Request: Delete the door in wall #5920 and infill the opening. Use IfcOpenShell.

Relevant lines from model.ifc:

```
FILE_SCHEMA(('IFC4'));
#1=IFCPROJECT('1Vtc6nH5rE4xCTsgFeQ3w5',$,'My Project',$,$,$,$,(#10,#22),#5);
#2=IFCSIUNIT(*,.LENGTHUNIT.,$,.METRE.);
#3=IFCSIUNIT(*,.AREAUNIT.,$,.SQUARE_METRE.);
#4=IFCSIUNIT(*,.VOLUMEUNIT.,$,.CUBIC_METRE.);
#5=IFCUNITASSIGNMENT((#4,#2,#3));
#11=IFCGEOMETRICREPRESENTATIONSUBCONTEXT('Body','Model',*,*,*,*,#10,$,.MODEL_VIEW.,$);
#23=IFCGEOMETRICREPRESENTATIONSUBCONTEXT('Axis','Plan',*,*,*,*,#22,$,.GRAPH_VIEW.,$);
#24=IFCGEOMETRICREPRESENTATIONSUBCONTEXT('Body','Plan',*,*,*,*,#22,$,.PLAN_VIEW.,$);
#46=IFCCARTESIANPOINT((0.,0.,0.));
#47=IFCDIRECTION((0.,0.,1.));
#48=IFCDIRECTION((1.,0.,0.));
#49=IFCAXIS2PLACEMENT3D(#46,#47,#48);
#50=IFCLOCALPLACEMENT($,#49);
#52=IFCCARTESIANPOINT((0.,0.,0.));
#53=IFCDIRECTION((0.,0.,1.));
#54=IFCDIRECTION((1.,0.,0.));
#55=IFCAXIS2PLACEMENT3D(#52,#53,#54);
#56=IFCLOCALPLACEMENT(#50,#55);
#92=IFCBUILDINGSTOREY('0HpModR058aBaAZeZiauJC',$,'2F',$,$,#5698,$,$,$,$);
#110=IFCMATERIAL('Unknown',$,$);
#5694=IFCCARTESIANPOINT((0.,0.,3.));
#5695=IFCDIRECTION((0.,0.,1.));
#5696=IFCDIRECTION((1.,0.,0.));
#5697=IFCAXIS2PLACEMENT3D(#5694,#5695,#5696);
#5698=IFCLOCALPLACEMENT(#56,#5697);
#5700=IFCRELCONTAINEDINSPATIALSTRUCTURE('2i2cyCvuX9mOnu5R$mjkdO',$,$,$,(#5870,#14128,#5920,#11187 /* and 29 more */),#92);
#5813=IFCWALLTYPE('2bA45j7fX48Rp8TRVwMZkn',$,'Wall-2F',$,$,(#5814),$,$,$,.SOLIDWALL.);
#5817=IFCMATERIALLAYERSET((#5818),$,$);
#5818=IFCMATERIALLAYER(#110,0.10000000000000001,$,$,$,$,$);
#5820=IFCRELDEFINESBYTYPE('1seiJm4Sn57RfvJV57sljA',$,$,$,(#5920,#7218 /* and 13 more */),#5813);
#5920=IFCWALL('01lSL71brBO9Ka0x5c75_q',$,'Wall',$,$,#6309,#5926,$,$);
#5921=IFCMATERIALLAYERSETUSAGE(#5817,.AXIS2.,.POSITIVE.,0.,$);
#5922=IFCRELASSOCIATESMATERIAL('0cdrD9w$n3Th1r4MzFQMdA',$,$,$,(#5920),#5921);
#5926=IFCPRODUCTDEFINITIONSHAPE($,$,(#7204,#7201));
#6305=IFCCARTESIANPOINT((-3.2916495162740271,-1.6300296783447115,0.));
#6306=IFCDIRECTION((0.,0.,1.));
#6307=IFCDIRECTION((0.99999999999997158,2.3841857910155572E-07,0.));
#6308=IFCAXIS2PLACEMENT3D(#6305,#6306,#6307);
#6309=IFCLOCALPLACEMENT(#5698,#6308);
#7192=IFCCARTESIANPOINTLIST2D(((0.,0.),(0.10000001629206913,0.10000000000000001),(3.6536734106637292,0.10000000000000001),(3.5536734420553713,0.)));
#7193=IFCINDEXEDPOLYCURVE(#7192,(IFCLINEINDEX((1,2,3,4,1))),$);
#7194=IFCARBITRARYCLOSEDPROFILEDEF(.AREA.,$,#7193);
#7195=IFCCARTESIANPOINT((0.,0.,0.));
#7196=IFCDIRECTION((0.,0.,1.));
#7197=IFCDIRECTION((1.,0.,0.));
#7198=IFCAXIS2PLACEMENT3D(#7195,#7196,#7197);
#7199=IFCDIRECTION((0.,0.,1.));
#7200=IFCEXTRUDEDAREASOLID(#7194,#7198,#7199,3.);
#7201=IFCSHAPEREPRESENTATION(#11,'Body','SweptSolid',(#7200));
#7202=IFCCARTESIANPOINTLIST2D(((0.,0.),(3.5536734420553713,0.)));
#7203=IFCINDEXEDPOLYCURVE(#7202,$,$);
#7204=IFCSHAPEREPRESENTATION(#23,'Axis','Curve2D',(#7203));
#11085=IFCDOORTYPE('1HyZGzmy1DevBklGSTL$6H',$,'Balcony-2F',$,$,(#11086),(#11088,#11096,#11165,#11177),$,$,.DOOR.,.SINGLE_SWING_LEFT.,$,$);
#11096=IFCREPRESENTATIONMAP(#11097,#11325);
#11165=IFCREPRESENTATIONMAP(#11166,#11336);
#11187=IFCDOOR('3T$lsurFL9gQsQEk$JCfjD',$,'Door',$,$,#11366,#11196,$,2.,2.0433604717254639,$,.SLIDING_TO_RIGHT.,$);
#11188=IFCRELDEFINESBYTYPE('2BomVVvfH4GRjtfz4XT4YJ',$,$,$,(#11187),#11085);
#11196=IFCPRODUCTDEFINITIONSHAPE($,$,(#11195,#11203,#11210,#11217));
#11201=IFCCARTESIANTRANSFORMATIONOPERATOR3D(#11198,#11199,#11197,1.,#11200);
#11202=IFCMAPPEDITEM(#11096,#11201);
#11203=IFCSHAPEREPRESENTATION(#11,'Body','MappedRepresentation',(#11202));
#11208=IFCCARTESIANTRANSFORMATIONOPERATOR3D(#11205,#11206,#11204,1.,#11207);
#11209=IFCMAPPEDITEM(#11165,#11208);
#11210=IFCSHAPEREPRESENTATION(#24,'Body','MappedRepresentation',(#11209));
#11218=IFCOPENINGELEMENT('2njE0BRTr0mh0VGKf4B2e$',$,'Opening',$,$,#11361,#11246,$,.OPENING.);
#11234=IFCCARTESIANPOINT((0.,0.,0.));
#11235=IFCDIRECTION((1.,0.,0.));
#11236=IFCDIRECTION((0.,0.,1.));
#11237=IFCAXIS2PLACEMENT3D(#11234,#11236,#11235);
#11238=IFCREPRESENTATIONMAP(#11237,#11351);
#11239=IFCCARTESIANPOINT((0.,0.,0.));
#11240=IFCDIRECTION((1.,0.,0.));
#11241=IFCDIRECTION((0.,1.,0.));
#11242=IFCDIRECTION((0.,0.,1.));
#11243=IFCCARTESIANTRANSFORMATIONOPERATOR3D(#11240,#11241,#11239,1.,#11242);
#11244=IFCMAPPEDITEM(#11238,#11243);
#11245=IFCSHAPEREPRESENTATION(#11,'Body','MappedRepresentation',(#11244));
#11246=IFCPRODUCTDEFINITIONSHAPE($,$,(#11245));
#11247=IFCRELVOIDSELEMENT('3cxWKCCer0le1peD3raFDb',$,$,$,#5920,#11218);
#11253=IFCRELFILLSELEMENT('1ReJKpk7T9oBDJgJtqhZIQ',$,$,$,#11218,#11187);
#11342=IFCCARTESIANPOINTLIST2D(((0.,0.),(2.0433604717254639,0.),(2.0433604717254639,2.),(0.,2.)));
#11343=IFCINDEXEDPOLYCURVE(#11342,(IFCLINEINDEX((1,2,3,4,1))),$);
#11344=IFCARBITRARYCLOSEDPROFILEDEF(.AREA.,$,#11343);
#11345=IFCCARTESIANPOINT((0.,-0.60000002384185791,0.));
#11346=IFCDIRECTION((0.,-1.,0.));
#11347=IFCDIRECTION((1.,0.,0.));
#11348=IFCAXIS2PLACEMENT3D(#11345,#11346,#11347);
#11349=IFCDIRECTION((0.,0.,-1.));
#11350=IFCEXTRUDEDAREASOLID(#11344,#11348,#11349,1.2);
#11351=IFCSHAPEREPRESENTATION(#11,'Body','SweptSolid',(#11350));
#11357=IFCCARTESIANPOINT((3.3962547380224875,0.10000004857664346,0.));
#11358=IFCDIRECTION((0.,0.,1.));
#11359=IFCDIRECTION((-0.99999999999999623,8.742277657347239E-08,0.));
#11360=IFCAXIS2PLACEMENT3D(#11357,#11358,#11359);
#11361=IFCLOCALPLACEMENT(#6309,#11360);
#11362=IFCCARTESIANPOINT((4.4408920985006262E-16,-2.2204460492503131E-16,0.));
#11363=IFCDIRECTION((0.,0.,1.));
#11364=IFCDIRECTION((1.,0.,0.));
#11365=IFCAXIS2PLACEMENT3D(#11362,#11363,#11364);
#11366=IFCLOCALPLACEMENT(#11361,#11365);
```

```python
import ifcopenshell
import ifcopenshell.api.feature
import ifcopenshell.api.root
import ifcopenshell.geom
import ifcopenshell.util.shape

model = ifcopenshell.open("model.ifc")
settings = ifcopenshell.geom.settings()


def volume(element):
    """Net volume in cubic metres, openings subtracted."""
    shape = ifcopenshell.geom.create_shape(settings, element)
    return ifcopenshell.util.shape.get_volume(shape.geometry)


door = model.by_guid("3T$lsurFL9gQsQEk$JCfjD")
opening = door.FillsVoids[0].RelatingOpeningElement
wall = opening.VoidsElements[0].RelatingBuildingElement
before = volume(wall)

ifcopenshell.api.root.remove_product(model, product=door)
ifcopenshell.api.feature.remove_feature(model, feature=opening)

after = volume(wall)

print(f"wall volume {before:.3f} -> {after:.3f} m3")

model.write("model_edited.ifc")
```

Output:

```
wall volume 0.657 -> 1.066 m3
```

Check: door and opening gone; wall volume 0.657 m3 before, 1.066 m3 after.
